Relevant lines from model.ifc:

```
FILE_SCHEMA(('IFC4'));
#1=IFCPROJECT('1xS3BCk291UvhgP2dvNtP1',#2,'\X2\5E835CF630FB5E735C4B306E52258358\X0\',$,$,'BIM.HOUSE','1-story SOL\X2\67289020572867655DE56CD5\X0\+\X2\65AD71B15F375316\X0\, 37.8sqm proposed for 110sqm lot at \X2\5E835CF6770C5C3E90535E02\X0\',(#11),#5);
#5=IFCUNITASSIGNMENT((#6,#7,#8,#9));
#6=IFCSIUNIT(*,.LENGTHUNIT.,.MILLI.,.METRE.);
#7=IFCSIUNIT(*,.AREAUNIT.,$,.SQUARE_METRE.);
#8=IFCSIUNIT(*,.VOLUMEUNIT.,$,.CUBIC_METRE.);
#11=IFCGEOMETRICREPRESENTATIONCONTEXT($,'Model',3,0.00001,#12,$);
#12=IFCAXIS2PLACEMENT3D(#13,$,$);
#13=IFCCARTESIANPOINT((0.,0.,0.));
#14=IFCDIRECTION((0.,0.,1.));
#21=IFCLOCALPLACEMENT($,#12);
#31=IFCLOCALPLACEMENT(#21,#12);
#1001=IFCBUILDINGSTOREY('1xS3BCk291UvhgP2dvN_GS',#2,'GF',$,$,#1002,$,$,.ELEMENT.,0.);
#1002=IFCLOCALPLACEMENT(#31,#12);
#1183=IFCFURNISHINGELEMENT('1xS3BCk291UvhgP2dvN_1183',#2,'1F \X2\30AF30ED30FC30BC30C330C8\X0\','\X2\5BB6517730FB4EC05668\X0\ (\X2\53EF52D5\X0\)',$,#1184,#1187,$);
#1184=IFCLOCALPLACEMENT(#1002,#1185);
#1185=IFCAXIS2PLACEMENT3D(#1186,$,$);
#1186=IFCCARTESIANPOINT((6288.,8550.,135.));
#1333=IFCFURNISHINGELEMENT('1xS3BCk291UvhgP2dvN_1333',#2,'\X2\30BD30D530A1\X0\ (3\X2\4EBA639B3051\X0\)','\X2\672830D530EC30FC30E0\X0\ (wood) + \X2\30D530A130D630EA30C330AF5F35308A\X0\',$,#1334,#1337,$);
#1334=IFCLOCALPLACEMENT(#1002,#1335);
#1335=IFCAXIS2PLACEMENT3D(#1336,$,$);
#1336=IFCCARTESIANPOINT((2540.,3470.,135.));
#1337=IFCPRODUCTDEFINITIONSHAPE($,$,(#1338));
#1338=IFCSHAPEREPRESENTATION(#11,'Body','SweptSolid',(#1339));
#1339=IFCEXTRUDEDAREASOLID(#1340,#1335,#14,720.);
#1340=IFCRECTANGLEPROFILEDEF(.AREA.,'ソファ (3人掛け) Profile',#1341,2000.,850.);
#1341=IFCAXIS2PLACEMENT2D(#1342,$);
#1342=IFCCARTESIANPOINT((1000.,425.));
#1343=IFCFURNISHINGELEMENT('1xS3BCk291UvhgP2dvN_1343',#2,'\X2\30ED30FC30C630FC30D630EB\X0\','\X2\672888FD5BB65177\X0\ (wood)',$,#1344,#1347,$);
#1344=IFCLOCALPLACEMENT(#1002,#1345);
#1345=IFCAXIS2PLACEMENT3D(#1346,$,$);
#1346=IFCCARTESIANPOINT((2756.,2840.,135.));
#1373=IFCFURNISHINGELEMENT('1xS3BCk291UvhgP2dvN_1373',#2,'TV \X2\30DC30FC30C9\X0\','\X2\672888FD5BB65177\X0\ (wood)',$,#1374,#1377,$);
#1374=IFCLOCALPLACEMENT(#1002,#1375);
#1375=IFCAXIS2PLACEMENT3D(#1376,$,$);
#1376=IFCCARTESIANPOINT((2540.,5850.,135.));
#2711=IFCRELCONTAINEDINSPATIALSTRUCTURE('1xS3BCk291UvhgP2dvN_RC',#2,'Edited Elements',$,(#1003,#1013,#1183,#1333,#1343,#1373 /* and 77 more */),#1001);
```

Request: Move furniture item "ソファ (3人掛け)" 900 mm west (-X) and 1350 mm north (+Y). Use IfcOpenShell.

```python
import ifcopenshell
import ifcopenshell.api.geometry
import ifcopenshell.util.placement
import ifcopenshell.util.unit

model = ifcopenshell.open("model.ifc")
unit_scale = ifcopenshell.util.unit.calculate_unit_scale(model)

item = model.by_guid("1xS3BCk291UvhgP2dvN_1333")
matrix = ifcopenshell.util.placement.get_local_placement(item.ObjectPlacement)
matrix[0, 3] -= 0.9 / unit_scale
matrix[1, 3] += 1.35 / unit_scale
ifcopenshell.api.geometry.edit_object_placement(model, product=item, matrix=matrix, is_si=False)

print(ifcopenshell.util.placement.get_local_placement(item.ObjectPlacement).round(3) + 0.0)

model.write("model_v2.ifc")
```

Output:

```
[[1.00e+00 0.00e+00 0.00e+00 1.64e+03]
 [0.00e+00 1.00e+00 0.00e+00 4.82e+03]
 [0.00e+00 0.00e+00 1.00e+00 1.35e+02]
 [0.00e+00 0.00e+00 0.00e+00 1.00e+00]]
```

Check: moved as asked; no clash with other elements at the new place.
